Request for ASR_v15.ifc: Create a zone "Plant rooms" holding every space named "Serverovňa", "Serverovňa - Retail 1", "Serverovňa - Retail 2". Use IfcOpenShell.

First a look at what the model holds.

```python
import ifcopenshell

model = ifcopenshell.open("ASR_v15.ifc")
print(model.schema)
seen = {}
for space in model.by_type("IfcSpace"):
    seen[space.LongName] = seen.get(space.LongName, 0) + 1
for name, count in sorted(seen.items(), key=str):
    print(count, "x", name)
print("zones:", [z.Name for z in model.by_type("IfcZone")][:20])
```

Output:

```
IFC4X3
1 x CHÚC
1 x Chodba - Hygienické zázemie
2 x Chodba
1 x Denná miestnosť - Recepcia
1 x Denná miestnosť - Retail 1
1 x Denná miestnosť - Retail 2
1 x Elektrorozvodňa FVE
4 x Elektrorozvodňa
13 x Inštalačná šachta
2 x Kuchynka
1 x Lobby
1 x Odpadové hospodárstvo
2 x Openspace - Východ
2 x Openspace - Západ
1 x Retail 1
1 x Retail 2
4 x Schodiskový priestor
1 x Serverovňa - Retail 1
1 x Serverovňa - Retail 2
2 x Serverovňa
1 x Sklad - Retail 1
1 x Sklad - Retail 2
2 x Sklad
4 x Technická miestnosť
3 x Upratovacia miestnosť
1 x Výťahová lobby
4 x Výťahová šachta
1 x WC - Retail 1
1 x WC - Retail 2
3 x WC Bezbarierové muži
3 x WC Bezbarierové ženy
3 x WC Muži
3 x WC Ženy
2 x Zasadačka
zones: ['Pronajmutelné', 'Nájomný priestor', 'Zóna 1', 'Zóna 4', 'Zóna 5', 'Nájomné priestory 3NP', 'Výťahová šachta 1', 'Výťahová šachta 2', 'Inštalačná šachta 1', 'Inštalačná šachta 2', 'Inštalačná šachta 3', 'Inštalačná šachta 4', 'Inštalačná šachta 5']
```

```python
import ifcopenshell
import ifcopenshell.api.group
import ifcopenshell.api.root

model = ifcopenshell.open("ASR_v15.ifc")

names = {"Serverovňa", "Serverovňa - Retail 1", "Serverovňa - Retail 2"}
spaces = [s for s in model.by_type("IfcSpace") if s.LongName in names]

zone = ifcopenshell.api.root.create_entity(model, ifc_class="IfcZone", name="Plant rooms")
ifcopenshell.api.group.assign_group(model, products=spaces, group=zone)
print(len(spaces), "spaces in", zone.Name)

model.write("ASR_v15_v2.ifc")
```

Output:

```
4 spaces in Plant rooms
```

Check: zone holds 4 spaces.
